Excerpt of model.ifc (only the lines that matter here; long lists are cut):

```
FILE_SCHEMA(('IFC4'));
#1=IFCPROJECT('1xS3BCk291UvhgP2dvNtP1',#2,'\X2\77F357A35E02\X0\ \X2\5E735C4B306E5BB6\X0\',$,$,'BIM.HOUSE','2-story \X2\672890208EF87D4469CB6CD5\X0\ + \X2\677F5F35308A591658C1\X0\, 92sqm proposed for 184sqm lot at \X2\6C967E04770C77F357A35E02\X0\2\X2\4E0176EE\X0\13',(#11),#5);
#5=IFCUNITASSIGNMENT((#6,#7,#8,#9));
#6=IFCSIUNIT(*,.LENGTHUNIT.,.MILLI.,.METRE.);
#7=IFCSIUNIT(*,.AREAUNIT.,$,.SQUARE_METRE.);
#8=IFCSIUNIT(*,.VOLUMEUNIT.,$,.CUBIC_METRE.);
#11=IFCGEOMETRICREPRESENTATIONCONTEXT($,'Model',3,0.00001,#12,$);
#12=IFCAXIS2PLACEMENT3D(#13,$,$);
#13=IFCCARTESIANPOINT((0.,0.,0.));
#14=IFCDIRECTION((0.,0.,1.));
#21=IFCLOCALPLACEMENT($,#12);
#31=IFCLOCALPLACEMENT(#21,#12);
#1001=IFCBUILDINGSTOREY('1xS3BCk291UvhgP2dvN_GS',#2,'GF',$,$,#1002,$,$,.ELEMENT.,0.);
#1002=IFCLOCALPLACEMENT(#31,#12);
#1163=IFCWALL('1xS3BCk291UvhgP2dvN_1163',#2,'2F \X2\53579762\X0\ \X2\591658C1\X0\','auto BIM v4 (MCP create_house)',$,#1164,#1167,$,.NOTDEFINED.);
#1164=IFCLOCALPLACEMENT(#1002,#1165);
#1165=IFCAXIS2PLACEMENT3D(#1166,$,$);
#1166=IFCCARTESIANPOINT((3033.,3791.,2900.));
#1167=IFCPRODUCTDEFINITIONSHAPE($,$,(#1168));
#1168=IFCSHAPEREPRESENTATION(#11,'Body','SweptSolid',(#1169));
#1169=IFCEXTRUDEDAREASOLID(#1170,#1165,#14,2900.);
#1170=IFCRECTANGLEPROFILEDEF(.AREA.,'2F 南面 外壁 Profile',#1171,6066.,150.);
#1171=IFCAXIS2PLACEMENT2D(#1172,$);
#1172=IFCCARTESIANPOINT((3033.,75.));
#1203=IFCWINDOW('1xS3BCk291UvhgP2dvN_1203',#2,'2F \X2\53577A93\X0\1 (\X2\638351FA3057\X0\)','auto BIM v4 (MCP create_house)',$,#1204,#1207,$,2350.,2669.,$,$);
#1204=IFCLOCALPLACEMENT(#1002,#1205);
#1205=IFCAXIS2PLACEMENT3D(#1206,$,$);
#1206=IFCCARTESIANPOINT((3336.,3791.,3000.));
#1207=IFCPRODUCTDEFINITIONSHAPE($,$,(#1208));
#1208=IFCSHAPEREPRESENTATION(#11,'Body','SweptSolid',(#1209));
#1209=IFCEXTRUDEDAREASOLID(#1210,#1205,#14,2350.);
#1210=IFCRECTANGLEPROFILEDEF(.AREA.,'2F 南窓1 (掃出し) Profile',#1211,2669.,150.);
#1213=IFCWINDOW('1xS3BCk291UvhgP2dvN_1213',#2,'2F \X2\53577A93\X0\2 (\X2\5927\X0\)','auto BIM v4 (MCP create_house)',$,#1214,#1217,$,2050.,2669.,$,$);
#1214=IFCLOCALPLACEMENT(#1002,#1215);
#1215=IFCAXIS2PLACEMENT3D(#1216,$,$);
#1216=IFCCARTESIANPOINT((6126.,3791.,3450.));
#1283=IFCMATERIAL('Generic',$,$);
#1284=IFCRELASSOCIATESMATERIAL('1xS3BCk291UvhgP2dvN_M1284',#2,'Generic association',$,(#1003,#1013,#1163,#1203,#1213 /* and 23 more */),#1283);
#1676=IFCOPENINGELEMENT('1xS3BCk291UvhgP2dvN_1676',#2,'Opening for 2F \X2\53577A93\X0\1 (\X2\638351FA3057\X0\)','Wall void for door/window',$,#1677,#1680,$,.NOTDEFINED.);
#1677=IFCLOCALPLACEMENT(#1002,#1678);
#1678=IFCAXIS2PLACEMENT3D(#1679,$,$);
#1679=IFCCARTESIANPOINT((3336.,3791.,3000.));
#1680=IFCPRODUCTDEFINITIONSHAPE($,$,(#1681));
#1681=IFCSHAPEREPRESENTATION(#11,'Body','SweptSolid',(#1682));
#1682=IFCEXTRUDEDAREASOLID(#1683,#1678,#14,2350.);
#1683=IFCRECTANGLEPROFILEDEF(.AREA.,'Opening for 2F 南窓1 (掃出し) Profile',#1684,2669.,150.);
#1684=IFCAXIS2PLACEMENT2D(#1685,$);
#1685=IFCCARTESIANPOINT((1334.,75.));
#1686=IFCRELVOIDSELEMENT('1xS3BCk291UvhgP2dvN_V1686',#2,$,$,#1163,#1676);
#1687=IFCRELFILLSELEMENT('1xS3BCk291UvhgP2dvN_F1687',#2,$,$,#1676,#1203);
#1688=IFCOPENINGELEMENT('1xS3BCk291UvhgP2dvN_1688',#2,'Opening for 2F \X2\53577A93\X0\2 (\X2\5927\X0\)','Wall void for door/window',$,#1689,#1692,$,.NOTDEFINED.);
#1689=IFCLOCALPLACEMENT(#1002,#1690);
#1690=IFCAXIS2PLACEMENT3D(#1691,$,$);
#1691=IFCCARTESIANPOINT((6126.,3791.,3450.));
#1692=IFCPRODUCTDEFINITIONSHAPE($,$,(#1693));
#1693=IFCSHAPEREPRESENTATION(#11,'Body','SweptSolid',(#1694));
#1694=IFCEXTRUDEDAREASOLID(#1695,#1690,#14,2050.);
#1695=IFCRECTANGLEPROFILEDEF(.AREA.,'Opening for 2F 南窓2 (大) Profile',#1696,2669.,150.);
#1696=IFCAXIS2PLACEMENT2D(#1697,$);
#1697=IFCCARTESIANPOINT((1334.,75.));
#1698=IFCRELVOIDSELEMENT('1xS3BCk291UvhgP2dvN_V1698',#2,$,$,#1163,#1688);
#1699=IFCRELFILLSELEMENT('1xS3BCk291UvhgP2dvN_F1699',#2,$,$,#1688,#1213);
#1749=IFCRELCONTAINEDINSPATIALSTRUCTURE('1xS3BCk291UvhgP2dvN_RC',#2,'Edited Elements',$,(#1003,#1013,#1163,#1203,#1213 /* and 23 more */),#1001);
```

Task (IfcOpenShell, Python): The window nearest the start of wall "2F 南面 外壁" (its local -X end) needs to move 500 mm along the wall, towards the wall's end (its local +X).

```python
import ifcopenshell
import ifcopenshell.api.geometry
import ifcopenshell.util.placement
import ifcopenshell.util.unit

model = ifcopenshell.open("model.ifc")
unit_scale = ifcopenshell.util.unit.calculate_unit_scale(model)

window = model.by_id(1203)
opening = window.FillsVoids[0].RelatingOpeningElement
wall = opening.VoidsElements[0].RelatingBuildingElement

wall_matrix = ifcopenshell.util.placement.get_local_placement(wall.ObjectPlacement)
shift = wall_matrix[:3, 0] * 0.5 / unit_scale
before = ifcopenshell.util.placement.get_local_placement(window.ObjectPlacement)[:3, 3].copy()

# The window is not placed relative to its opening, so move both.
for product in (opening, window):
    matrix = ifcopenshell.util.placement.get_local_placement(product.ObjectPlacement)
    matrix[:3, 3] += shift
    ifcopenshell.api.geometry.edit_object_placement(model, product=product, matrix=matrix, is_si=False)

after = ifcopenshell.util.placement.get_local_placement(window.ObjectPlacement)[:3, 3]
print("window moved by", (after - before).round(3) + 0.0)

model.write("model_edited.ifc")
```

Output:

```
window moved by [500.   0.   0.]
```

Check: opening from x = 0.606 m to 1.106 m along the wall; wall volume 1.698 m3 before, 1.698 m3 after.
